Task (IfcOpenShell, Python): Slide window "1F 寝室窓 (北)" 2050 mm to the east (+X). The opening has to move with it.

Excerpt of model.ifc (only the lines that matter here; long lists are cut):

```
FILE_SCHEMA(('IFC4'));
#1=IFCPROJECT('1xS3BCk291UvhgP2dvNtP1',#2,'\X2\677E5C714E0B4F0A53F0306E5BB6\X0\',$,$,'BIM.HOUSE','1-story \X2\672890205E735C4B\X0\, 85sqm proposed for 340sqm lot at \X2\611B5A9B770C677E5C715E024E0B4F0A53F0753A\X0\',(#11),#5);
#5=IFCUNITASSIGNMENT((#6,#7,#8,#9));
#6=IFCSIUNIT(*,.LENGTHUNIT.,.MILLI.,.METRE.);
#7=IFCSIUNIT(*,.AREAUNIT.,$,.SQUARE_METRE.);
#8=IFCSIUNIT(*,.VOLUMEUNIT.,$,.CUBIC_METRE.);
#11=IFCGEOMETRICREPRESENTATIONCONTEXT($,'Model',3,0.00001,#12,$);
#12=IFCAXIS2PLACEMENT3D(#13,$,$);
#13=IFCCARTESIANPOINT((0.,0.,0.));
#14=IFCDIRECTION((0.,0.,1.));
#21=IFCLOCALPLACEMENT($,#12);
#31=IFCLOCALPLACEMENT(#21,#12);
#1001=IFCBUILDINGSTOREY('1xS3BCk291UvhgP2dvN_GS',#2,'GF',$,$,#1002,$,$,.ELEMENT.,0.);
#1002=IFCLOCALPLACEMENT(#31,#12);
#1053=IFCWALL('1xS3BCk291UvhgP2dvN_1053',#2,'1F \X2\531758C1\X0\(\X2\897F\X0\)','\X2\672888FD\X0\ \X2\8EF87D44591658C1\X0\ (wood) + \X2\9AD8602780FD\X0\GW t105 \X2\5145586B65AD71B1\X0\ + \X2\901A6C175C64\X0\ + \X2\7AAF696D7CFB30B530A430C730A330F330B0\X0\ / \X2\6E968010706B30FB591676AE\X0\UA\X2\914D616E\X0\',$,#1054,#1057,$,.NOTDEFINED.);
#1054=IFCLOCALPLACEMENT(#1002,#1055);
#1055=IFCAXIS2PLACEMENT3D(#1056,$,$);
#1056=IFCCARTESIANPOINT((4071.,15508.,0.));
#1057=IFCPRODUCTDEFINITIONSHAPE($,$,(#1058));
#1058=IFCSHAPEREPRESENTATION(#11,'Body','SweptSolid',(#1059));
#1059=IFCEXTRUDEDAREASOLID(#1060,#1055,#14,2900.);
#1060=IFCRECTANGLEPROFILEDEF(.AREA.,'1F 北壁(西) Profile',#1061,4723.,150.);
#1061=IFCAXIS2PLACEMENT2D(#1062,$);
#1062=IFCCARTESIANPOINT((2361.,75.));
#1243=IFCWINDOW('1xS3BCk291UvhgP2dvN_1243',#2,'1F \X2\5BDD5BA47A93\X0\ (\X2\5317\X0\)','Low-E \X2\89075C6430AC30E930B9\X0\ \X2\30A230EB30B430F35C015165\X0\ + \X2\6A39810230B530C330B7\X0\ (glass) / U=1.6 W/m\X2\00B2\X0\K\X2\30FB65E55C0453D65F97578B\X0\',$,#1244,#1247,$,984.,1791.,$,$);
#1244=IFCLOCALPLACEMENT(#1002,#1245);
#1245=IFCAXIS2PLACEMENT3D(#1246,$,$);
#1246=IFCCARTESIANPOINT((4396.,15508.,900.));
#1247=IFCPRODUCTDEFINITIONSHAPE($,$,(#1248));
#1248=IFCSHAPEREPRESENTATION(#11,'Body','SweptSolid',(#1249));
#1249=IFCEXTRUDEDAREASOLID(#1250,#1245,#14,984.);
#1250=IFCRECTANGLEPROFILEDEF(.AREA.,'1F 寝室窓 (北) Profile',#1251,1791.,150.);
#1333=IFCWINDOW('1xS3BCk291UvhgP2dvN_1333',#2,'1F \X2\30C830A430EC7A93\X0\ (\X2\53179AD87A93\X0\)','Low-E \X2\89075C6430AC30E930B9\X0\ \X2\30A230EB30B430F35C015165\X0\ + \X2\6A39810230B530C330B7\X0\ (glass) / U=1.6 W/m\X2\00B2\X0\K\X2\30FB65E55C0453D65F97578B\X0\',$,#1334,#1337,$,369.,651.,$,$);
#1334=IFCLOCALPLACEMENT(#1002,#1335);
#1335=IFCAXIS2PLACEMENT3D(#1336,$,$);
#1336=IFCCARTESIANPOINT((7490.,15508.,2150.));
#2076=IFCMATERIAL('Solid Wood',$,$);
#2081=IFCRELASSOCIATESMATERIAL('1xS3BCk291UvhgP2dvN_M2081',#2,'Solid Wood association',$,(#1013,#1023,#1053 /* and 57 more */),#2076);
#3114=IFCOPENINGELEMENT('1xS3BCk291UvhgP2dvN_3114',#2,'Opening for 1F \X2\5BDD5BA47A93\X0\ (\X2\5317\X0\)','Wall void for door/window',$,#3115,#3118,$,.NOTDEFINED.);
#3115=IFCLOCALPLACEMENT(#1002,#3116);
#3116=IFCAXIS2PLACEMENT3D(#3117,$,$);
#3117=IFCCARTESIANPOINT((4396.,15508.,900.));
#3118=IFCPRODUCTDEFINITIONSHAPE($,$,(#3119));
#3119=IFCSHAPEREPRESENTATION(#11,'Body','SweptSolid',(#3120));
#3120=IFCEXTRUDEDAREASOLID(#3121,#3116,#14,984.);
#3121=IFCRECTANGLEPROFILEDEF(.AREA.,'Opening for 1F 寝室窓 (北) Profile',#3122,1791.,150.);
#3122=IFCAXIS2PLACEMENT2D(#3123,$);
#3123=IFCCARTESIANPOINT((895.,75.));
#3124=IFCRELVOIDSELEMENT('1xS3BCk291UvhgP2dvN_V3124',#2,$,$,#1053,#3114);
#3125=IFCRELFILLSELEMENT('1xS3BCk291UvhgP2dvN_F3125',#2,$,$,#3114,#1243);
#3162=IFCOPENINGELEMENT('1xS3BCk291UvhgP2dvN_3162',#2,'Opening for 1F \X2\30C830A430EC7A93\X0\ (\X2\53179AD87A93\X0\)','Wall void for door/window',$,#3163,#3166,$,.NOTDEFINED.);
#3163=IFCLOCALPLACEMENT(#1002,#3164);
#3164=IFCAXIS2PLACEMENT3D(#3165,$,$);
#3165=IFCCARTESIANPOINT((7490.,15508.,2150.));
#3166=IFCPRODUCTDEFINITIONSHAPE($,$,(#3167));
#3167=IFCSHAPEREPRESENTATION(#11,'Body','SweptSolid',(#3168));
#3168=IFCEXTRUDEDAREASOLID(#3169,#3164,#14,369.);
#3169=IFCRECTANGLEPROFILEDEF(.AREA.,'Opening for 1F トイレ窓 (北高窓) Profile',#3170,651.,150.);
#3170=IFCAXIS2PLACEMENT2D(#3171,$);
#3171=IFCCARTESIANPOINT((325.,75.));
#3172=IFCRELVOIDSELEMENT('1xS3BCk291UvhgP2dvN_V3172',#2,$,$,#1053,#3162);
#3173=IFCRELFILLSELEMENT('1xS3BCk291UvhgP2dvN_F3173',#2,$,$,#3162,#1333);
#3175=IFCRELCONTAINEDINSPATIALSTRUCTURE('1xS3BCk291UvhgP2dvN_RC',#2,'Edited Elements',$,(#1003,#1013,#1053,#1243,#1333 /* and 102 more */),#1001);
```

```python
import ifcopenshell
import ifcopenshell.api.geometry
import ifcopenshell.util.placement
import ifcopenshell.util.unit

model = ifcopenshell.open("model.ifc")
unit_scale = ifcopenshell.util.unit.calculate_unit_scale(model)

window = model.by_guid("1xS3BCk291UvhgP2dvN_1243")
opening = window.FillsVoids[0].RelatingOpeningElement
wall = opening.VoidsElements[0].RelatingBuildingElement

wall_matrix = ifcopenshell.util.placement.get_local_placement(wall.ObjectPlacement)
shift = wall_matrix[:3, 0] * 2.05 / unit_scale
before = ifcopenshell.util.placement.get_local_placement(window.ObjectPlacement)[:3, 3].copy()

# The window is not placed relative to its opening, so move both.
for product in (opening, window):
    matrix = ifcopenshell.util.placement.get_local_placement(product.ObjectPlacement)
    matrix[:3, 3] += shift
    ifcopenshell.api.geometry.edit_object_placement(model, product=product, matrix=matrix, is_si=False)

after = ifcopenshell.util.placement.get_local_placement(window.ObjectPlacement)[:3, 3]
print("window moved by", (after - before).round(3) + 0.0)

model.write("model_rev.ifc")
```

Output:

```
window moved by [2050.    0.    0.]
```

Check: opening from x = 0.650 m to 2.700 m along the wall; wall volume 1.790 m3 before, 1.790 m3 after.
